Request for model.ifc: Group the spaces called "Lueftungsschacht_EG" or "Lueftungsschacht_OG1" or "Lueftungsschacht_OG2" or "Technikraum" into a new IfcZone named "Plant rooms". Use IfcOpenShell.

First a look at what the model holds.

```python
import ifcopenshell

model = ifcopenshell.open("model.ifc")
print(model.schema)
seen = {}
for space in model.by_type("IfcSpace"):
    seen[space.LongName] = seen.get(space.LongName, 0) + 1
for name, count in sorted(seen.items(), key=str):
    print(count, "x", name)
print("zones:", [z.Name for z in model.by_type("IfcZone")][:20])
```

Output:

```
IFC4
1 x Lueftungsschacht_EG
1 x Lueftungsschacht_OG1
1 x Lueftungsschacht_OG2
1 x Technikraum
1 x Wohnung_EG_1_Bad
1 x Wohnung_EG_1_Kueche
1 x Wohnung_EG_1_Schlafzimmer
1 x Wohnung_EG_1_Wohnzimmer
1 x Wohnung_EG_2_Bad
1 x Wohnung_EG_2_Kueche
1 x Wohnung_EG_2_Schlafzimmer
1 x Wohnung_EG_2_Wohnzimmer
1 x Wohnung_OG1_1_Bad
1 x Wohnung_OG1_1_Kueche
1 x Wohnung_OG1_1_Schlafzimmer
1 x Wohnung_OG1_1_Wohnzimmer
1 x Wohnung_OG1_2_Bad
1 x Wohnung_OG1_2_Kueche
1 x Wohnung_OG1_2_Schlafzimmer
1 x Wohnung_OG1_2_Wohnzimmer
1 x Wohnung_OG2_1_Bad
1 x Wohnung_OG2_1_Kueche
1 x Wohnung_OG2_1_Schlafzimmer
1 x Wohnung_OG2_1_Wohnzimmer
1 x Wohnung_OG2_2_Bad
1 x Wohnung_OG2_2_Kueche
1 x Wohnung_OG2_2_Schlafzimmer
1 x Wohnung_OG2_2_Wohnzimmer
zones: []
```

```python
import ifcopenshell
import ifcopenshell.api.group
import ifcopenshell.api.root

model = ifcopenshell.open("model.ifc")

names = {"Lueftungsschacht_EG", "Lueftungsschacht_OG1", "Lueftungsschacht_OG2", "Technikraum"}
spaces = [s for s in model.by_type("IfcSpace") if s.LongName in names]

zone = ifcopenshell.api.root.create_entity(model, ifc_class="IfcZone", name="Plant rooms")
ifcopenshell.api.group.assign_group(model, products=spaces, group=zone)
print(len(spaces), "spaces in", zone.Name)

model.write("model-out.ifc")
```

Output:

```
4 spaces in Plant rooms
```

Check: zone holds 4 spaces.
